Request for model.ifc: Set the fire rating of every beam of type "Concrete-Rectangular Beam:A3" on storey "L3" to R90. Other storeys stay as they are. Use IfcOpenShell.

First a look at what the model holds.

```python
import ifcopenshell
import ifcopenshell.util.element

model = ifcopenshell.open("model.ifc")
print(model.schema)
storey = next(s for s in model.by_type("IfcBuildingStorey") if s.Name == "L3")
beams = [e for e in ifcopenshell.util.element.get_decomposition(storey) if e.is_a("IfcBeam")]
seen = {}
for e in beams:
    element_type = ifcopenshell.util.element.get_type(e)
    key = (element_type.Name if element_type != e and element_type else None, ifcopenshell.util.element.get_pset(e, "Pset_BeamCommon", "FireRating"))
    seen[key] = seen.get(key, 0) + 1
for (name, value), count in sorted(seen.items(), key=str):
    print(count, "x", name, "|", value)
```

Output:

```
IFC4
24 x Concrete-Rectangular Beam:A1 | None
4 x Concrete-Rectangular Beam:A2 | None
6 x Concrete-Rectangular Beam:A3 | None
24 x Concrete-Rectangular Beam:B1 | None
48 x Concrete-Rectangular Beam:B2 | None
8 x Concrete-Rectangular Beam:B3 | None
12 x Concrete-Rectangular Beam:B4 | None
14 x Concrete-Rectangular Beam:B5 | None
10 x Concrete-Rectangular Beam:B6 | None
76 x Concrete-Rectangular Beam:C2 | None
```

```python
import ifcopenshell
import ifcopenshell.api.pset
import ifcopenshell.util.element

model = ifcopenshell.open("model.ifc")

storey = next(s for s in model.by_type("IfcBuildingStorey") if s.Name == "L3")
beams = [e for e in ifcopenshell.util.element.get_decomposition(storey) if e.is_a("IfcBeam")]

count = 0
for e in beams:
    element_type = ifcopenshell.util.element.get_type(e)
    if element_type in (None, e) or element_type.Name != "Concrete-Rectangular Beam:A3":
        continue
    # add_pset returns the element's existing set when there is one.
    pset = ifcopenshell.api.pset.add_pset(model, product=e, name="Pset_BeamCommon")
    ifcopenshell.api.pset.edit_pset(model, pset=pset, properties={"FireRating": "R90"})
    count += 1

print(count, "beams updated")

model.write("model-out.ifc")
```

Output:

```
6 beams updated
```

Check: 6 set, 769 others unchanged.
